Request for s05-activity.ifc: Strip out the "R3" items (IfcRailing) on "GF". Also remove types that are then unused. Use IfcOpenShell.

First a look at what the model holds.

```python
import ifcopenshell
import ifcopenshell.util.element

model = ifcopenshell.open("s05-activity.ifc")
print(model.schema)
storey = next(s for s in model.by_type("IfcBuildingStorey") if s.Name == "GF")
railings = [e for e in ifcopenshell.util.element.get_decomposition(storey) if e.is_a("IfcRailing")]
seen = {}
for e in railings:
    element_type = ifcopenshell.util.element.get_type(e)
    name = element_type.Name if element_type not in (None, e) else None
    seen[name] = seen.get(name, 0) + 1
for name, count in sorted(seen.items(), key=str):
    print(count, "x", name)
```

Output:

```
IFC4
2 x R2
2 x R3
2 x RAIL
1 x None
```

```python
import ifcopenshell
import ifcopenshell.api.root
import ifcopenshell.util.element

model = ifcopenshell.open("s05-activity.ifc")

storey = next(s for s in model.by_type("IfcBuildingStorey") if s.Name == "GF")
railings = [e for e in ifcopenshell.util.element.get_decomposition(storey) if e.is_a("IfcRailing")]
targets = [e for e in railings if (t := ifcopenshell.util.element.get_type(e)) not in (None, e) and t.Name == "R3"]
types = {ifcopenshell.util.element.get_type(e) for e in targets} - {None, *targets}

for e in targets:
    ifcopenshell.api.root.remove_product(model, product=e)
print(len(targets), "removed")

unused = [t for t in types if not ifcopenshell.util.element.get_types(t)]
for t in unused:
    ifcopenshell.api.root.remove_product(model, product=t)
print(len(unused), "unused types removed")

model.write("s05-activity_updated.ifc")
```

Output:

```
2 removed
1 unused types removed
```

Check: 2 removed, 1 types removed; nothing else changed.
